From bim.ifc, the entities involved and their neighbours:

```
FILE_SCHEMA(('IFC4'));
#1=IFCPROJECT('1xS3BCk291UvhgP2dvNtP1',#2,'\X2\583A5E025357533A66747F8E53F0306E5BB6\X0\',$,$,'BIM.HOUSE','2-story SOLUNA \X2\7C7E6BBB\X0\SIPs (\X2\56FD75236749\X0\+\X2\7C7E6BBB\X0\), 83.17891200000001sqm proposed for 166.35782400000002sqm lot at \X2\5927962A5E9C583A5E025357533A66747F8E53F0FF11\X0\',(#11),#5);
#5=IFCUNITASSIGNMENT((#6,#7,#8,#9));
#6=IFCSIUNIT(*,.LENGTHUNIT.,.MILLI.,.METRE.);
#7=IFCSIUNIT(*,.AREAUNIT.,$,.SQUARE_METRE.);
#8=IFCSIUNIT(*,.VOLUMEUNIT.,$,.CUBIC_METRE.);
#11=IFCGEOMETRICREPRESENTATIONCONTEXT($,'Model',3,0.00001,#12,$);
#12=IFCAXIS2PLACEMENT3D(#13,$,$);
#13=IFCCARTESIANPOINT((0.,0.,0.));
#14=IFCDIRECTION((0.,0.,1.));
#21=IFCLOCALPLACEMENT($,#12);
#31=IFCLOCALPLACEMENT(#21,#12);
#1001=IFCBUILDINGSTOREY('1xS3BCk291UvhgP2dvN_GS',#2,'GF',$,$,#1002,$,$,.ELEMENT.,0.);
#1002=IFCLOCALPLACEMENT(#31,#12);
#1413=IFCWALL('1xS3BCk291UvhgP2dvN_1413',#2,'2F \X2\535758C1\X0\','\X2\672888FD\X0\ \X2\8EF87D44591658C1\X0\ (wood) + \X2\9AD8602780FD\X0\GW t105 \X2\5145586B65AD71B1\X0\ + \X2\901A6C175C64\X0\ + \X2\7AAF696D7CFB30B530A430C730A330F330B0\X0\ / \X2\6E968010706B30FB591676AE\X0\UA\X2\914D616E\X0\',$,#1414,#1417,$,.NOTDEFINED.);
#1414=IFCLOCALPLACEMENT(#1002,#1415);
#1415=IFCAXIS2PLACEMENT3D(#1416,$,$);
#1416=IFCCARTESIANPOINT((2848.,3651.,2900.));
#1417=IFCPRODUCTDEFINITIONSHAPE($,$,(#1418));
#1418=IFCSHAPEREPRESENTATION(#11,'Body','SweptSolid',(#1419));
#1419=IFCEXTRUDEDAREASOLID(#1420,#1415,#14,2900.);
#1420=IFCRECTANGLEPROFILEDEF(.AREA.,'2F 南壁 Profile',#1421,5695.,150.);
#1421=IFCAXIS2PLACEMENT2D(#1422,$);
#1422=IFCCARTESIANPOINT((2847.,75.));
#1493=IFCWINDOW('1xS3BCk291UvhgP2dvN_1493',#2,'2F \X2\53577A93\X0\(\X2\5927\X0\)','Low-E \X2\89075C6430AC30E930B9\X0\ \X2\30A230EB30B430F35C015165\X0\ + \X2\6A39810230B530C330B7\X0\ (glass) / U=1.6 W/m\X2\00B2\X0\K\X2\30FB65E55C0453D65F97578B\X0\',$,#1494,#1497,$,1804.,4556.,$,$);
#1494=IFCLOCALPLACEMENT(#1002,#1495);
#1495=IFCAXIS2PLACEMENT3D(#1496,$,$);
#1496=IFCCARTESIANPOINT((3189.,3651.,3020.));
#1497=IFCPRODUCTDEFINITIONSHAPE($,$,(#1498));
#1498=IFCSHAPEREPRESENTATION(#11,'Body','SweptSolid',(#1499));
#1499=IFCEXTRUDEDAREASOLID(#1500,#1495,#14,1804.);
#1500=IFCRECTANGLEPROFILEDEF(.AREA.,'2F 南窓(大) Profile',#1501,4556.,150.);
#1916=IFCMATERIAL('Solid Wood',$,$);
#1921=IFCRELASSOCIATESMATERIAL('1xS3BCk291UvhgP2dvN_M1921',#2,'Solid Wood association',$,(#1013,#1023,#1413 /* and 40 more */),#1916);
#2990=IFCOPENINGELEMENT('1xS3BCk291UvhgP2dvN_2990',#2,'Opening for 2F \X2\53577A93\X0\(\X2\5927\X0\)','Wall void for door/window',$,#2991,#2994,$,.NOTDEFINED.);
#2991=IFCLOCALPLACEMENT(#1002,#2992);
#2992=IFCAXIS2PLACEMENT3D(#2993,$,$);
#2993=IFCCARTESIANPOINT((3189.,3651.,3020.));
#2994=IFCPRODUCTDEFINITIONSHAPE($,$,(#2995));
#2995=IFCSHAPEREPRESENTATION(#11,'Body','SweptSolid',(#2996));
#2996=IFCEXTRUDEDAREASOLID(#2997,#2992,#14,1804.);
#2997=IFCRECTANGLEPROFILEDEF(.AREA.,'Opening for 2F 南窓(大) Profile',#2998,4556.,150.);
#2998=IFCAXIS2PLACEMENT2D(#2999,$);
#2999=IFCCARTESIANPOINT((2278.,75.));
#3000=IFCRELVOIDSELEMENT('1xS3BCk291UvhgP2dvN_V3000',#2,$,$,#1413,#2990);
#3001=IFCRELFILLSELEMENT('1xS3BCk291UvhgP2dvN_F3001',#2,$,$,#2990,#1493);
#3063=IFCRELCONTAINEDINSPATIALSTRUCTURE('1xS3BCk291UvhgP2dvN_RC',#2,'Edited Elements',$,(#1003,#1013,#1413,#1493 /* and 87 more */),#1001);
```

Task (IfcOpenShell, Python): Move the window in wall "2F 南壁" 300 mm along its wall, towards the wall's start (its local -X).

```python
import ifcopenshell
import ifcopenshell.api.geometry
import ifcopenshell.util.placement
import ifcopenshell.util.unit

model = ifcopenshell.open("bim.ifc")
unit_scale = ifcopenshell.util.unit.calculate_unit_scale(model)

window = model.by_id(1493)
opening = window.FillsVoids[0].RelatingOpeningElement
wall = opening.VoidsElements[0].RelatingBuildingElement

wall_matrix = ifcopenshell.util.placement.get_local_placement(wall.ObjectPlacement)
shift = wall_matrix[:3, 0] * -0.3 / unit_scale
before = ifcopenshell.util.placement.get_local_placement(window.ObjectPlacement)[:3, 3].copy()

# The window is not placed relative to its opening, so move both.
for product in (opening, window):
    matrix = ifcopenshell.util.placement.get_local_placement(product.ObjectPlacement)
    matrix[:3, 3] += shift
    ifcopenshell.api.geometry.edit_object_placement(model, product=product, matrix=matrix, is_si=False)

after = ifcopenshell.util.placement.get_local_placement(window.ObjectPlacement)[:3, 3]
print("window moved by", (after - before).round(3) + 0.0)

model.write("bim_v2.ifc")
```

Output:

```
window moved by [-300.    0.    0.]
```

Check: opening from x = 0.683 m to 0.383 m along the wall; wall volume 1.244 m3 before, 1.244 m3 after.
